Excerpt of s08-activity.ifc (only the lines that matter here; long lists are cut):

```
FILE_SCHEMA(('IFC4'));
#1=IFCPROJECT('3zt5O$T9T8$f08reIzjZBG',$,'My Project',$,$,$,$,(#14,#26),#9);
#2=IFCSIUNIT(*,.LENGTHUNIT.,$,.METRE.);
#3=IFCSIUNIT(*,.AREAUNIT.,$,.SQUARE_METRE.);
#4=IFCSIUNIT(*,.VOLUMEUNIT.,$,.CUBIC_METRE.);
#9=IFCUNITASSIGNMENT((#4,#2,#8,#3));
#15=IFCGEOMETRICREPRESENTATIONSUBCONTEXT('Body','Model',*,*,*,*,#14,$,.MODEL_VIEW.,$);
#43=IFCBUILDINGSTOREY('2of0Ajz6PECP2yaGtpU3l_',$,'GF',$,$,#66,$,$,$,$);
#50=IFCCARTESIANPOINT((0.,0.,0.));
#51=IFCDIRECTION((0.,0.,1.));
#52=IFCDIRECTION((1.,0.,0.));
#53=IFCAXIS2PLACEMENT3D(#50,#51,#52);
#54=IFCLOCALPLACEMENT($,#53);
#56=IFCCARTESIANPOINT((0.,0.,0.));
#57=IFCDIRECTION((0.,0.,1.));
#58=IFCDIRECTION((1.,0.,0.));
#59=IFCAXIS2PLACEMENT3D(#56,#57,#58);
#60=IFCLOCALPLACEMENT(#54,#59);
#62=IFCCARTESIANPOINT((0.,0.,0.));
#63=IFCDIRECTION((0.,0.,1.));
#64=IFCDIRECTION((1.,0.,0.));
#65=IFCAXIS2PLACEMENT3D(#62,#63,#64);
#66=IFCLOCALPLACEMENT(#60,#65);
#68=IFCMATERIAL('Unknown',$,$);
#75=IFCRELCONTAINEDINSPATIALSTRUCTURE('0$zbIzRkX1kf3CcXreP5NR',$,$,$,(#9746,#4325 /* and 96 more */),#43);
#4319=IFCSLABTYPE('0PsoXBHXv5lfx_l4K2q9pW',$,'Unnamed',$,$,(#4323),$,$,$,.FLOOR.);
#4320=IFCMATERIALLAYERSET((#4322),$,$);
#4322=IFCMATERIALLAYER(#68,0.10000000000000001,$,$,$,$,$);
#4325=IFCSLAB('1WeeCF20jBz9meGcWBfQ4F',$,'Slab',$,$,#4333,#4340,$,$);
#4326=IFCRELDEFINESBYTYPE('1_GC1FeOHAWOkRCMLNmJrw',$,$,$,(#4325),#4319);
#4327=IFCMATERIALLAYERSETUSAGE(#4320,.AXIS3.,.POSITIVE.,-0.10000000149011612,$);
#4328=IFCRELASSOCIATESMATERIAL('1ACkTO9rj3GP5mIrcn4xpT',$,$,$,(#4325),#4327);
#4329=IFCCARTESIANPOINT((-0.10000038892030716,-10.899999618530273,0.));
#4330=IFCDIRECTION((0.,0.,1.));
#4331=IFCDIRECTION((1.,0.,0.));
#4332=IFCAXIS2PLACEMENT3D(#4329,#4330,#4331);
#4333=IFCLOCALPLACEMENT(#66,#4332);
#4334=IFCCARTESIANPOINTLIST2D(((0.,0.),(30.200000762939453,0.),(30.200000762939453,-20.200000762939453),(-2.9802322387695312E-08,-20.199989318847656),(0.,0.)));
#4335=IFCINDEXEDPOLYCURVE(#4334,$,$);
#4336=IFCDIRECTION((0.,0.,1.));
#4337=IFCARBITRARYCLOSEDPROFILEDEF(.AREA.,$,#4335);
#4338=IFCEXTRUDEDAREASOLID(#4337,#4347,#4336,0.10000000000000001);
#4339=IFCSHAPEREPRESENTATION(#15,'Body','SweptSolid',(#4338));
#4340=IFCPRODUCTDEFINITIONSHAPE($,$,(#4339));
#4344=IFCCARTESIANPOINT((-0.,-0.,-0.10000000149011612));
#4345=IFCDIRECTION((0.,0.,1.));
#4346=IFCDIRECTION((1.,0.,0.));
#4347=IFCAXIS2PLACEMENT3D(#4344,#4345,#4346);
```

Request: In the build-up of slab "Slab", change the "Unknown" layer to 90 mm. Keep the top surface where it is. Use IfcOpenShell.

```python
import ifcopenshell
import ifcopenshell.util.element
import ifcopenshell.util.representation
import ifcopenshell.util.unit

model = ifcopenshell.open("s08-activity.ifc")
unit_scale = ifcopenshell.util.unit.calculate_unit_scale(model)

layer_set = model.by_id(4320)
layer = next(l for l in layer_set.MaterialLayers if l.Material and l.Material.Name == "Unknown")
change = 0.09 / unit_scale - layer.LayerThickness
layer.LayerThickness += change

# Geometry does not follow the layer set by itself.
slabs = [e for e in ifcopenshell.util.element.get_elements_by_material(model, layer_set) if e.is_a("IfcSlab")]
for slab in sorted(slabs, key=lambda e: e.id()):
    body = ifcopenshell.util.representation.get_representation(slab, "Model", "Body")
    solid = body.Items[0]
    old_depth = solid.Depth
    solid.Depth += change
    # Extruded upwards: lower the start of the extrusion so the top stays.
    x, y, z = solid.Position.Location.Coordinates
    solid.Position.Location = model.createIfcCartesianPoint((x, y, z - change))
    print(slab.id(), f"{old_depth:g} -> {solid.Depth:g}")

# The layers are counted up from the underside, which has moved.
for usage in {ifcopenshell.util.element.get_material(slab) for slab in slabs}:
    usage.OffsetFromReferenceLine -= change

model.write("s08-activity-out.ifc")
```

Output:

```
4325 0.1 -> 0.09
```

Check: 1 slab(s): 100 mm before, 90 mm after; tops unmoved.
